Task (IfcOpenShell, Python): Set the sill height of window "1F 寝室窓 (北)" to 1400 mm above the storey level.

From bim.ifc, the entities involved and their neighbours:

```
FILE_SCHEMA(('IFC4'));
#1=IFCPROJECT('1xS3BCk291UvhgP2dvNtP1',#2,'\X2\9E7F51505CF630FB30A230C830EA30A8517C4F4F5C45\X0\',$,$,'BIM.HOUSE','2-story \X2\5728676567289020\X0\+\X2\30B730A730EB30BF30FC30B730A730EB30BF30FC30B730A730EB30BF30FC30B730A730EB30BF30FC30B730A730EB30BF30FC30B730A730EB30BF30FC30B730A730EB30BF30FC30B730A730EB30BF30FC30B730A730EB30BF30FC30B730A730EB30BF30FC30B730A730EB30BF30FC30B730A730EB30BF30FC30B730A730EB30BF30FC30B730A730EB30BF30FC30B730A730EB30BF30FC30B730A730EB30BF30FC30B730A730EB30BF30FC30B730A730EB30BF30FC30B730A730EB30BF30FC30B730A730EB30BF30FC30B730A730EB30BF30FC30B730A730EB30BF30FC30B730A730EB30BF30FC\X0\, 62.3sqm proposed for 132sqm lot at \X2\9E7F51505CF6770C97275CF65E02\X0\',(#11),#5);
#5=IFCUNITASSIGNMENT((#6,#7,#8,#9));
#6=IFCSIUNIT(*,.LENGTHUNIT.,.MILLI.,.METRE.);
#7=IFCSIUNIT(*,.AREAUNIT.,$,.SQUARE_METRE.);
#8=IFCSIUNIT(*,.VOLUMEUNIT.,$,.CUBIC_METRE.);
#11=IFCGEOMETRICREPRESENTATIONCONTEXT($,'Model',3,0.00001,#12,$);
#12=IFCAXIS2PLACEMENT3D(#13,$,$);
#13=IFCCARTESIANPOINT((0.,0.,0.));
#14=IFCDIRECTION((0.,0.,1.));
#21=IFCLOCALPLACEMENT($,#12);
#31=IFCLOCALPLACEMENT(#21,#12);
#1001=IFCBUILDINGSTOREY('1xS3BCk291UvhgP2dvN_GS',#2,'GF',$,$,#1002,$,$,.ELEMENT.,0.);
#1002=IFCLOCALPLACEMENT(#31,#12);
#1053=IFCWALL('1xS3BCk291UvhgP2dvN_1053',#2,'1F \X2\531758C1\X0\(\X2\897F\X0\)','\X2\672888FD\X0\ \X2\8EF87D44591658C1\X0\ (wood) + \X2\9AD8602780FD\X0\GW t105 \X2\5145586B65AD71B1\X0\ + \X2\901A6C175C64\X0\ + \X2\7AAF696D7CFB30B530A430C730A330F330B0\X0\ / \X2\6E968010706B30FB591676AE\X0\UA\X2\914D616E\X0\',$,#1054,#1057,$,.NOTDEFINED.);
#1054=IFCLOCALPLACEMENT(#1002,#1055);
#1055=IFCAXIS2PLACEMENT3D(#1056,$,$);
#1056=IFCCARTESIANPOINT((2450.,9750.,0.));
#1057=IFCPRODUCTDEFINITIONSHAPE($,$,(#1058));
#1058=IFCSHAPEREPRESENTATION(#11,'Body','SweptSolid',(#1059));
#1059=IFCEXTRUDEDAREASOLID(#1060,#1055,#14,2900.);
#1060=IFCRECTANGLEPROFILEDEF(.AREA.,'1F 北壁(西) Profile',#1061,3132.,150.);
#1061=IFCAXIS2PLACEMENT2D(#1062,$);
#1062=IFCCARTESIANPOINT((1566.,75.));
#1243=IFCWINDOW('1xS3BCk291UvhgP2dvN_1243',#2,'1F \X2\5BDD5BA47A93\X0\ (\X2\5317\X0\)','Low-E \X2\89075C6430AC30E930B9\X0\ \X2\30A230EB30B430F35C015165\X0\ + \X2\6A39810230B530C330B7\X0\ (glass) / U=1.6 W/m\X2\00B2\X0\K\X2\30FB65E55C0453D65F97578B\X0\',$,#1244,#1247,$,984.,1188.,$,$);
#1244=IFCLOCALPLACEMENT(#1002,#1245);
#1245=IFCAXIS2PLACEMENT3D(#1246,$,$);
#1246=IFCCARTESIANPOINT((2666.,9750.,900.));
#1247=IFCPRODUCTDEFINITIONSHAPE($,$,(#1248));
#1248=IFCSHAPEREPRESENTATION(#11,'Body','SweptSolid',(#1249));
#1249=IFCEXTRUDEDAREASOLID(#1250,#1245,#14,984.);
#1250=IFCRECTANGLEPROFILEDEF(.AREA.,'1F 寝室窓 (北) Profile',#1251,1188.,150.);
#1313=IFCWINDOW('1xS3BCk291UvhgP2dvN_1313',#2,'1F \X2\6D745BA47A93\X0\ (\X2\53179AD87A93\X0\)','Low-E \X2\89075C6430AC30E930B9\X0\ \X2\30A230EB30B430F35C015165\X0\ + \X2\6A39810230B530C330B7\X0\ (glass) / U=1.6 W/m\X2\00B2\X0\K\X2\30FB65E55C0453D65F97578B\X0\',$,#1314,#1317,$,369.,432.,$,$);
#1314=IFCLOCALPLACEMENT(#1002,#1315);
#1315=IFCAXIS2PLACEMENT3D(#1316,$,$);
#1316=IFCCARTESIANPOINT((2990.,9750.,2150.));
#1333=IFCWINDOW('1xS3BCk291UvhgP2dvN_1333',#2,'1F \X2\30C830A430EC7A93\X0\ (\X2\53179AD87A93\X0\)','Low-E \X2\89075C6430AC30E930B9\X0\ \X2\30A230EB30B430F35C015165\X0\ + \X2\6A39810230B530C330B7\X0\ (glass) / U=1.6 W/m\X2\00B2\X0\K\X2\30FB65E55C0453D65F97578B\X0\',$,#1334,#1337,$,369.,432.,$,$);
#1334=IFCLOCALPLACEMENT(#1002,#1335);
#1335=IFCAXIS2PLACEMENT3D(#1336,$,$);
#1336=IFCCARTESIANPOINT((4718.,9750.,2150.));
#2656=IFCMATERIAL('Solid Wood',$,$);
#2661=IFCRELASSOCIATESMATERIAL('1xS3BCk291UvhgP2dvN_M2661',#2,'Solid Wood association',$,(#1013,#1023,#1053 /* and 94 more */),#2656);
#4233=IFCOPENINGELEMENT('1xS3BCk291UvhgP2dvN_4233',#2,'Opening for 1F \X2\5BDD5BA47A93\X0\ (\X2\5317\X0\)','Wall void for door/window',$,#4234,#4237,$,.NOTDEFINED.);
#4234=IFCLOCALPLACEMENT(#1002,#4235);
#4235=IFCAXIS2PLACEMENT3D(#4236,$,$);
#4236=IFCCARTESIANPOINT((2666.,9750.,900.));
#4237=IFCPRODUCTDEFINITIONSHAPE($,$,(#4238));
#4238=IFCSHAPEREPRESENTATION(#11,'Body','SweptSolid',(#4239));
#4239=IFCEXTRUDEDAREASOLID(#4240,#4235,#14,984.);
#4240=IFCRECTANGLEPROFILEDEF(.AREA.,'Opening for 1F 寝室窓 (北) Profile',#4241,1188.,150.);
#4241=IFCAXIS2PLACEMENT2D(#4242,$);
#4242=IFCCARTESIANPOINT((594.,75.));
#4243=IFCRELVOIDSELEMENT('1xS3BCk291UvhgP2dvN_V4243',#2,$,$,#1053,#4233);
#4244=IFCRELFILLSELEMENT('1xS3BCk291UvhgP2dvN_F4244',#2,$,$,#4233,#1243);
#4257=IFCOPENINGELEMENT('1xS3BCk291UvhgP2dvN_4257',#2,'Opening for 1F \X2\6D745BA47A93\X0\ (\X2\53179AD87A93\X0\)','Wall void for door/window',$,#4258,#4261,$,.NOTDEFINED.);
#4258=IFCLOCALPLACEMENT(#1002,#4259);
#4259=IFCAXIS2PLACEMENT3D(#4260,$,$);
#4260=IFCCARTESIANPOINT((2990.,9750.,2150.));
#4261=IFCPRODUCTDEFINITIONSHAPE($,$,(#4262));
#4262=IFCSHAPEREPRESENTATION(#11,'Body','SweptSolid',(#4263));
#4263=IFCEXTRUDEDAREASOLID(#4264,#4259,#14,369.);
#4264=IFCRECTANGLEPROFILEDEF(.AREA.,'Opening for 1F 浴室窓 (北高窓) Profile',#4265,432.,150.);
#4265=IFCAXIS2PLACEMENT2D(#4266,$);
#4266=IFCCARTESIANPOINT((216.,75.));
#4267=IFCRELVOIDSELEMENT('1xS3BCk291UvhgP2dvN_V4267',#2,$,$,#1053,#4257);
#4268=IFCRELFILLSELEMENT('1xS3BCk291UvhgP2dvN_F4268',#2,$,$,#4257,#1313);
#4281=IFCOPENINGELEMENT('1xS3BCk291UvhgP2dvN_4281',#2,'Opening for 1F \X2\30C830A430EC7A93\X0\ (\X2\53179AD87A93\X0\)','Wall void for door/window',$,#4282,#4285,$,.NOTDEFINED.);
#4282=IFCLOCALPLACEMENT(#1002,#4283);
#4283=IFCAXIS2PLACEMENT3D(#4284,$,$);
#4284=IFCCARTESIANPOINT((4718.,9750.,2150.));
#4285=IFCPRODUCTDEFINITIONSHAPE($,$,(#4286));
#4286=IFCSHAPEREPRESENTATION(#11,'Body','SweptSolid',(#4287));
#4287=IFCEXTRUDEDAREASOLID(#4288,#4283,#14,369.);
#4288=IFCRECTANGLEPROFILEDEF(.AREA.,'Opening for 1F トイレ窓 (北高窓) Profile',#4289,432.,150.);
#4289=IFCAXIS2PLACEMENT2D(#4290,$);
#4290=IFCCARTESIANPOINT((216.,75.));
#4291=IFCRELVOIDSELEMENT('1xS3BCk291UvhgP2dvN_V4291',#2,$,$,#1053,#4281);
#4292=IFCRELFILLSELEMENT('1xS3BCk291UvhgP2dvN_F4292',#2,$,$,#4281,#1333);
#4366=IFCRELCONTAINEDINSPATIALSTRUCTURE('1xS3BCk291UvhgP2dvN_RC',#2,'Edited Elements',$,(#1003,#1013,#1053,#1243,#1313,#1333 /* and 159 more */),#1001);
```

```python
import numpy as np
import ifcopenshell
import ifcopenshell.api.geometry
import ifcopenshell.geom
import ifcopenshell.util.element
import ifcopenshell.util.placement
import ifcopenshell.util.shape
import ifcopenshell.util.unit

model = ifcopenshell.open("bim.ifc")
unit_scale = ifcopenshell.util.unit.calculate_unit_scale(model)

window = model.by_guid("1xS3BCk291UvhgP2dvN_1243")
opening = window.FillsVoids[0].RelatingOpeningElement
storey = ifcopenshell.util.element.get_container(window, ifc_class="IfcBuildingStorey")
level = ifcopenshell.util.placement.get_local_placement(storey.ObjectPlacement)[2, 3]

# The opening's origin need not be at the sill, so measure its lowest point.
shape = ifcopenshell.geom.create_shape(ifcopenshell.geom.settings(), opening)
bottom = ifcopenshell.util.shape.get_shape_bottom_elevation(shape, shape.geometry) / unit_scale
dz = level + 1.4 / unit_scale - bottom

shift = np.array([0.0, 0.0, dz])
# The window is not placed relative to its opening, so move both.
for product in (opening, window):
    matrix = ifcopenshell.util.placement.get_local_placement(product.ObjectPlacement)
    matrix[:3, 3] += shift
    ifcopenshell.api.geometry.edit_object_placement(model, product=product, matrix=matrix, is_si=False)

print(f"moved by {dz * unit_scale:+.3f} m")

model.write("bim_edited.ifc")
```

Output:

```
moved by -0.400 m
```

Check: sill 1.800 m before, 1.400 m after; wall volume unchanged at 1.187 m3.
